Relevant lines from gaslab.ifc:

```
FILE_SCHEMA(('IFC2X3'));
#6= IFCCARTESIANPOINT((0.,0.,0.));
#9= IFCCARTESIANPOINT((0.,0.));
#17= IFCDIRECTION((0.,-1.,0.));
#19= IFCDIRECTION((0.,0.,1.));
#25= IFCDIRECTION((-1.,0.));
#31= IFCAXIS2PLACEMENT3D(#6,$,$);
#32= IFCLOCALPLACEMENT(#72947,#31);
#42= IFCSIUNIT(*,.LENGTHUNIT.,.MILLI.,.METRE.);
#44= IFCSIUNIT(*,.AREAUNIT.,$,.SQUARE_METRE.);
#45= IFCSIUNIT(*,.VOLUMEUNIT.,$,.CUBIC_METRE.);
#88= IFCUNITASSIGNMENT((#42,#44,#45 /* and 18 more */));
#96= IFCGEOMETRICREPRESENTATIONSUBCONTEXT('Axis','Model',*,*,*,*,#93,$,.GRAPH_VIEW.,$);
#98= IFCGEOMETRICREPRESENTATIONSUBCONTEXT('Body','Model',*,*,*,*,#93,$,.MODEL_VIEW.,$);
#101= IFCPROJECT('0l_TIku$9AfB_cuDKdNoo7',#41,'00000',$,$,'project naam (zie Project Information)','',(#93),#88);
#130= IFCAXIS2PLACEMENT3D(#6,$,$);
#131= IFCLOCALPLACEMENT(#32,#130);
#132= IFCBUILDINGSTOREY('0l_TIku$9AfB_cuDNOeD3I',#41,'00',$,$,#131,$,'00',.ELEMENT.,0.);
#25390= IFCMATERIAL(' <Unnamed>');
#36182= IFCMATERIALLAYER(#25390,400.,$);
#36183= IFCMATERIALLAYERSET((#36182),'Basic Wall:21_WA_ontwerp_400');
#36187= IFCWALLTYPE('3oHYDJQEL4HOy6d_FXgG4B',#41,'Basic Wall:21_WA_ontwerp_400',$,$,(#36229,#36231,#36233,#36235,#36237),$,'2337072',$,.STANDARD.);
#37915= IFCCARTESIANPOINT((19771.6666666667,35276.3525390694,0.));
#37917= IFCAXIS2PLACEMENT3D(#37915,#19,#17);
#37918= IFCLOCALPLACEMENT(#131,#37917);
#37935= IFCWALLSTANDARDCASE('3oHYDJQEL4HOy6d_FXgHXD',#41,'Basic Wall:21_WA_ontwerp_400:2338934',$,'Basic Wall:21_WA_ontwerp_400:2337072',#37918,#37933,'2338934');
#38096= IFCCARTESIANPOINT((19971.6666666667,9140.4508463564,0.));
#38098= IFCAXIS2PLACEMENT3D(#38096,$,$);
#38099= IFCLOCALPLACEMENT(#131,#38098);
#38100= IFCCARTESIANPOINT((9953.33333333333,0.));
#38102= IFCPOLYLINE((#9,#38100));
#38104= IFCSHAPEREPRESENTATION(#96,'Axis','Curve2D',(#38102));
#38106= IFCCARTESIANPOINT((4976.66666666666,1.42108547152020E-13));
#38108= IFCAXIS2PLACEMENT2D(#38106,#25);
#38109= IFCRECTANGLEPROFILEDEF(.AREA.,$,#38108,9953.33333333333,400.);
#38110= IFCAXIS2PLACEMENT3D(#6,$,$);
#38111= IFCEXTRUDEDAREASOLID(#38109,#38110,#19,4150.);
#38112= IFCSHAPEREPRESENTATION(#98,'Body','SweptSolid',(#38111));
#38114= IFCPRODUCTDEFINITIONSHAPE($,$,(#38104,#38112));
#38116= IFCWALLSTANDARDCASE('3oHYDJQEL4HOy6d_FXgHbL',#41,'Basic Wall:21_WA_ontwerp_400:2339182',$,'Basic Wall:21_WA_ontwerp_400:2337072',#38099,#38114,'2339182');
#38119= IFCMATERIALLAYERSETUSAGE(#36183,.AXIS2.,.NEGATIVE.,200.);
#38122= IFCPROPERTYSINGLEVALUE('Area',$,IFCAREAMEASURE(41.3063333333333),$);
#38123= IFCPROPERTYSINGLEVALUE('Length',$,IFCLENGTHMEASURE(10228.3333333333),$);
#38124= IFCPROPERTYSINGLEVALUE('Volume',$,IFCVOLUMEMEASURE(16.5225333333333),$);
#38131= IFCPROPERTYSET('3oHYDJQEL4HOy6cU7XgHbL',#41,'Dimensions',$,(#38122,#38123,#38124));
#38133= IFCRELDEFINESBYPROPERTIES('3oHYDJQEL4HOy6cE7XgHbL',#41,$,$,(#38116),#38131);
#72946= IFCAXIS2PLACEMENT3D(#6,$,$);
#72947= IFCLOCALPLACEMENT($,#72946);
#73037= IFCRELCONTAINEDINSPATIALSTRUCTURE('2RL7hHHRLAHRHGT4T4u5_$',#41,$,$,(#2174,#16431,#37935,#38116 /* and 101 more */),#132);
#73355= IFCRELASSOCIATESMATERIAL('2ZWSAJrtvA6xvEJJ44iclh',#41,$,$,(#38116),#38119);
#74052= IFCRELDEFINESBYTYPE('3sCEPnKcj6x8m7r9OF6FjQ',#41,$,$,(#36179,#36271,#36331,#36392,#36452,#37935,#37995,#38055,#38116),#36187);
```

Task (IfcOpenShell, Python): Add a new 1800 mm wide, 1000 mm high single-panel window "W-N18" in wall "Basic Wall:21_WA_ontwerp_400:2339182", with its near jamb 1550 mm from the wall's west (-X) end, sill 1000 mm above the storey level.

```python
import numpy as np
import ifcopenshell
import ifcopenshell.api.feature
import ifcopenshell.api.geometry
import ifcopenshell.api.pset
import ifcopenshell.api.root
import ifcopenshell.api.spatial
import ifcopenshell.api.type
import ifcopenshell.geom
import ifcopenshell.util.element
import ifcopenshell.util.placement
import ifcopenshell.util.representation
import ifcopenshell.util.shape
import ifcopenshell.util.unit

model = ifcopenshell.open("gaslab.ifc")
unit_scale = ifcopenshell.util.unit.calculate_unit_scale(model)
area_scale = ifcopenshell.util.unit.calculate_unit_scale(model, "AREAUNIT")
volume_scale = ifcopenshell.util.unit.calculate_unit_scale(model, "VOLUMEUNIT")
settings = ifcopenshell.geom.settings()


def volume(element):
    """Net volume in cubic metres, openings subtracted."""
    shape = ifcopenshell.geom.create_shape(settings, element)
    return ifcopenshell.util.shape.get_volume(shape.geometry)


wall = model.by_guid("3oHYDJQEL4HOy6d_FXgHbL")
storey = ifcopenshell.util.element.get_container(wall, ifc_class="IfcBuildingStorey")
context = ifcopenshell.util.representation.get_context(model, "Model", "Body", "MODEL_VIEW")
before = volume(wall)

width, height, from_end, sill = 1.8, 1, 1.55, 1  # metres

# The wall runs along its own X axis, and the end named is its -X end.
wall_shape = ifcopenshell.geom.create_shape(settings, wall)
x, y, z = ifcopenshell.util.shape.get_vertices(wall_shape.geometry).T
start = x.min() + from_end
face, thickness = float(y.min()), float(y.max() - y.min())
wall_matrix = ifcopenshell.util.placement.get_local_placement(wall.ObjectPlacement)
level = ifcopenshell.util.placement.get_local_placement(storey.ObjectPlacement)[2, 3]


def in_wall(x, y):
    """Placement at x, y metres in the wall's axes, at sill height."""
    matrix = wall_matrix.copy()
    matrix[:, 3] = wall_matrix @ np.array([x / unit_scale, y / unit_scale, 0.0, 1.0])
    matrix[2, 3] = level + sill / unit_scale
    return matrix


# Opening: a box that overshoots both wall faces by 50 mm.
opening = ifcopenshell.api.root.create_entity(model, ifc_class="IfcOpeningElement")
box = ifcopenshell.api.geometry.add_wall_representation(
    model, context=context, length=width, height=height, thickness=thickness + 0.1
)
ifcopenshell.api.geometry.assign_representation(model, product=opening, representation=box)
ifcopenshell.api.geometry.edit_object_placement(model, product=opening, matrix=in_wall(start, face - 0.05), is_si=False)
ifcopenshell.api.feature.add_feature(model, feature=opening, element=wall)

window = ifcopenshell.api.root.create_entity(model, ifc_class="IfcWindow", name="W-N18")
window.OverallWidth, window.OverallHeight = width / unit_scale, height / unit_scale
body = ifcopenshell.api.geometry.add_window_representation(
    model,
    context=context,
    overall_width=window.OverallWidth,
    overall_height=window.OverallHeight,
    partition_type="SINGLE_PANEL",
)
ifcopenshell.api.geometry.assign_representation(model, product=window, representation=body)
ifcopenshell.api.spatial.assign_container(model, products=[window], relating_structure=storey)
fills = ifcopenshell.api.feature.add_filling(model, opening=opening, element=window)
fills.OwnerHistory = window.OwnerHistory  # required in IFC2X3

# IFC2X3 keeps the operation on the window style.
style = ifcopenshell.api.root.create_entity(model, ifc_class="IfcWindowStyle", name="W-N18")
style.OperationType, style.ConstructionType = "SINGLE_PANEL", "NOTDEFINED"
style.ParameterTakesPrecedence = style.Sizeable = False
ifcopenshell.api.type.assign_type(model, related_objects=[window], relating_type=style)

# Centre the window in the wall's thickness.
ifcopenshell.api.geometry.edit_object_placement(model, product=window, matrix=in_wall(start, face), is_si=False)
window_shape = ifcopenshell.geom.create_shape(settings, window)
depth = ifcopenshell.util.shape.get_vertices(window_shape.geometry)[:, 1]
offset = face + thickness / 2 - (depth.min() + depth.max()) / 2
ifcopenshell.api.geometry.edit_object_placement(model, product=window, matrix=in_wall(start, offset), is_si=False)

after = volume(wall)

# Update the wall's stored quantities.
pset = model.by_id(ifcopenshell.util.element.get_pset(wall, "Dimensions", should_inherit=False)["id"])
ifcopenshell.api.pset.edit_pset(model, pset=pset, properties={
    "Area": model.create_entity("IfcAreaMeasure", after / thickness / area_scale),
    "Volume": model.create_entity("IfcVolumeMeasure", after / volume_scale),
})

print(f"wall volume {before:.3f} -> {after:.3f} m3")

model.write("gaslab_v2.ifc")
```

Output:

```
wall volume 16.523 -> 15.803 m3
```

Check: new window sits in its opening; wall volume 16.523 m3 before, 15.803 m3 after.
